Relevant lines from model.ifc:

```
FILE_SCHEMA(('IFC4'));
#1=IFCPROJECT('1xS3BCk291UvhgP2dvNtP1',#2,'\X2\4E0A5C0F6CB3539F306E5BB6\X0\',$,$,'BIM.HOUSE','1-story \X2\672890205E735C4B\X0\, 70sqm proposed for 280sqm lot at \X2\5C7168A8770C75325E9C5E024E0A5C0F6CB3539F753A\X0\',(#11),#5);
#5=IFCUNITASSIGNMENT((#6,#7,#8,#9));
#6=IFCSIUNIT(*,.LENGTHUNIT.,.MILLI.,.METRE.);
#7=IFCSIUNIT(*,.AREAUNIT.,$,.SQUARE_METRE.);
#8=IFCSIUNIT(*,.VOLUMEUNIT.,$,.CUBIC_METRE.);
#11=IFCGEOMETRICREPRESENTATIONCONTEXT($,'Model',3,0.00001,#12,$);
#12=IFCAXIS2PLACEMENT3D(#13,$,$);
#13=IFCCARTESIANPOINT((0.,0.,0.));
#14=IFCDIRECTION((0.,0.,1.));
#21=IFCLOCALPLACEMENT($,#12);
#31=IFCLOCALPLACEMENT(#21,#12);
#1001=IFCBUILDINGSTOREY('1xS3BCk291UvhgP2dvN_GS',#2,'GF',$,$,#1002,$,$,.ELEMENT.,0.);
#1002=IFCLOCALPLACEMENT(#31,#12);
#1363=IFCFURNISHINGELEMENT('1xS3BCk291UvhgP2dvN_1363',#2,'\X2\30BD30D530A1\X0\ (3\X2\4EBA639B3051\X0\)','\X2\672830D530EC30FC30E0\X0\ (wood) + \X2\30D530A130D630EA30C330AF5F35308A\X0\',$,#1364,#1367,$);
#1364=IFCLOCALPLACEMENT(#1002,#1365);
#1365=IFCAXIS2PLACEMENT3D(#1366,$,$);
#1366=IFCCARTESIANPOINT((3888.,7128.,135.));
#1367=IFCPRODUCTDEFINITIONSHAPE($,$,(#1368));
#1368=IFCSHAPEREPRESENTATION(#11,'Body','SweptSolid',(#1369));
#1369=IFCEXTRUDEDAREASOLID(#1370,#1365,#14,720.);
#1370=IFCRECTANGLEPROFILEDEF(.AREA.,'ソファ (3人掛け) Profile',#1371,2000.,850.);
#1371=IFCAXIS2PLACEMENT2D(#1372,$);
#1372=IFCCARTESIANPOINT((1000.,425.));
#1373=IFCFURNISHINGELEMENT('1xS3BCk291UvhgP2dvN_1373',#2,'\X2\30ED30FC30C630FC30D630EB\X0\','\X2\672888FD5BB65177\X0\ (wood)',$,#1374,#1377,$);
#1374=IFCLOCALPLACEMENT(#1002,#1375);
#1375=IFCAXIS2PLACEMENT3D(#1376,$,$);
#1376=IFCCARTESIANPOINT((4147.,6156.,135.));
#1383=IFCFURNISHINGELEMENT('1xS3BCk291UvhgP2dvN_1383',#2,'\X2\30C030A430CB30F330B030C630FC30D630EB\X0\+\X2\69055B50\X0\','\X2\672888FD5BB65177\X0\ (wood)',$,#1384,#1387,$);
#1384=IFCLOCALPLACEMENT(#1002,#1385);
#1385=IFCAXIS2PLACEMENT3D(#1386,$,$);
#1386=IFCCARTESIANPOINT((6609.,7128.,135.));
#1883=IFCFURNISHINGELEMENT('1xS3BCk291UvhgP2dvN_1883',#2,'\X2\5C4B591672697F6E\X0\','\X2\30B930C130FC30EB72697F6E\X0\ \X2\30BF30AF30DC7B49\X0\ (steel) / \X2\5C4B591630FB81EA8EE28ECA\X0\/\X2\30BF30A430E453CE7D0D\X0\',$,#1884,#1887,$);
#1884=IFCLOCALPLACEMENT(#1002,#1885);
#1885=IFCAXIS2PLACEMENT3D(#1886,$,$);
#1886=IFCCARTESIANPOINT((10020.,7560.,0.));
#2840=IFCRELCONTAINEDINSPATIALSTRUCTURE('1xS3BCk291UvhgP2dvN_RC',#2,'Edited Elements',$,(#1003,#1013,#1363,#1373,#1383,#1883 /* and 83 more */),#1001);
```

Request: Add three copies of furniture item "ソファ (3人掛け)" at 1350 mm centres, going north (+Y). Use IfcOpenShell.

```python
import numpy as np
import ifcopenshell
import ifcopenshell.api.geometry
import ifcopenshell.api.root
import ifcopenshell.util.element
import ifcopenshell.util.placement
import ifcopenshell.util.unit

model = ifcopenshell.open("model.ifc")
unit_scale = ifcopenshell.util.unit.calculate_unit_scale(model)


def reuse_history(source, copy):
    """copy_class also copies each property set's owner history, people and application; keep the originals."""
    for rel in copy.IsDefinedBy:
        if rel.is_a("IfcRelDefinesByProperties") and (history := rel.RelatingPropertyDefinition.OwnerHistory):
            rel.RelatingPropertyDefinition.OwnerHistory = source.OwnerHistory
            ifcopenshell.util.element.remove_deep2(model, history)


source = model.by_id(1363)
base = ifcopenshell.util.placement.get_local_placement(source.ObjectPlacement)
step = np.array([0.0, 1.0, 0.0]) * 1.35 / unit_scale

for i in range(1, 4):
    copy = ifcopenshell.api.root.copy_class(model, product=source)
    copy.Representation = ifcopenshell.util.element.copy_deep(
        model, source.Representation, exclude=["IfcGeometricRepresentationContext", "IfcRepresentationMap"]
    )
    reuse_history(source, copy)
    matrix = base.copy()
    matrix[:3, 3] += i * step
    print("added at", matrix[:3, 3].round(3) + 0.0)
    ifcopenshell.api.geometry.edit_object_placement(model, product=copy, matrix=matrix, is_si=False)

model.write("model_rev.ifc")
```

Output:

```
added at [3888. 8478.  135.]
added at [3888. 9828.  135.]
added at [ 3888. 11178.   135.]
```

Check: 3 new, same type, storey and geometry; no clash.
